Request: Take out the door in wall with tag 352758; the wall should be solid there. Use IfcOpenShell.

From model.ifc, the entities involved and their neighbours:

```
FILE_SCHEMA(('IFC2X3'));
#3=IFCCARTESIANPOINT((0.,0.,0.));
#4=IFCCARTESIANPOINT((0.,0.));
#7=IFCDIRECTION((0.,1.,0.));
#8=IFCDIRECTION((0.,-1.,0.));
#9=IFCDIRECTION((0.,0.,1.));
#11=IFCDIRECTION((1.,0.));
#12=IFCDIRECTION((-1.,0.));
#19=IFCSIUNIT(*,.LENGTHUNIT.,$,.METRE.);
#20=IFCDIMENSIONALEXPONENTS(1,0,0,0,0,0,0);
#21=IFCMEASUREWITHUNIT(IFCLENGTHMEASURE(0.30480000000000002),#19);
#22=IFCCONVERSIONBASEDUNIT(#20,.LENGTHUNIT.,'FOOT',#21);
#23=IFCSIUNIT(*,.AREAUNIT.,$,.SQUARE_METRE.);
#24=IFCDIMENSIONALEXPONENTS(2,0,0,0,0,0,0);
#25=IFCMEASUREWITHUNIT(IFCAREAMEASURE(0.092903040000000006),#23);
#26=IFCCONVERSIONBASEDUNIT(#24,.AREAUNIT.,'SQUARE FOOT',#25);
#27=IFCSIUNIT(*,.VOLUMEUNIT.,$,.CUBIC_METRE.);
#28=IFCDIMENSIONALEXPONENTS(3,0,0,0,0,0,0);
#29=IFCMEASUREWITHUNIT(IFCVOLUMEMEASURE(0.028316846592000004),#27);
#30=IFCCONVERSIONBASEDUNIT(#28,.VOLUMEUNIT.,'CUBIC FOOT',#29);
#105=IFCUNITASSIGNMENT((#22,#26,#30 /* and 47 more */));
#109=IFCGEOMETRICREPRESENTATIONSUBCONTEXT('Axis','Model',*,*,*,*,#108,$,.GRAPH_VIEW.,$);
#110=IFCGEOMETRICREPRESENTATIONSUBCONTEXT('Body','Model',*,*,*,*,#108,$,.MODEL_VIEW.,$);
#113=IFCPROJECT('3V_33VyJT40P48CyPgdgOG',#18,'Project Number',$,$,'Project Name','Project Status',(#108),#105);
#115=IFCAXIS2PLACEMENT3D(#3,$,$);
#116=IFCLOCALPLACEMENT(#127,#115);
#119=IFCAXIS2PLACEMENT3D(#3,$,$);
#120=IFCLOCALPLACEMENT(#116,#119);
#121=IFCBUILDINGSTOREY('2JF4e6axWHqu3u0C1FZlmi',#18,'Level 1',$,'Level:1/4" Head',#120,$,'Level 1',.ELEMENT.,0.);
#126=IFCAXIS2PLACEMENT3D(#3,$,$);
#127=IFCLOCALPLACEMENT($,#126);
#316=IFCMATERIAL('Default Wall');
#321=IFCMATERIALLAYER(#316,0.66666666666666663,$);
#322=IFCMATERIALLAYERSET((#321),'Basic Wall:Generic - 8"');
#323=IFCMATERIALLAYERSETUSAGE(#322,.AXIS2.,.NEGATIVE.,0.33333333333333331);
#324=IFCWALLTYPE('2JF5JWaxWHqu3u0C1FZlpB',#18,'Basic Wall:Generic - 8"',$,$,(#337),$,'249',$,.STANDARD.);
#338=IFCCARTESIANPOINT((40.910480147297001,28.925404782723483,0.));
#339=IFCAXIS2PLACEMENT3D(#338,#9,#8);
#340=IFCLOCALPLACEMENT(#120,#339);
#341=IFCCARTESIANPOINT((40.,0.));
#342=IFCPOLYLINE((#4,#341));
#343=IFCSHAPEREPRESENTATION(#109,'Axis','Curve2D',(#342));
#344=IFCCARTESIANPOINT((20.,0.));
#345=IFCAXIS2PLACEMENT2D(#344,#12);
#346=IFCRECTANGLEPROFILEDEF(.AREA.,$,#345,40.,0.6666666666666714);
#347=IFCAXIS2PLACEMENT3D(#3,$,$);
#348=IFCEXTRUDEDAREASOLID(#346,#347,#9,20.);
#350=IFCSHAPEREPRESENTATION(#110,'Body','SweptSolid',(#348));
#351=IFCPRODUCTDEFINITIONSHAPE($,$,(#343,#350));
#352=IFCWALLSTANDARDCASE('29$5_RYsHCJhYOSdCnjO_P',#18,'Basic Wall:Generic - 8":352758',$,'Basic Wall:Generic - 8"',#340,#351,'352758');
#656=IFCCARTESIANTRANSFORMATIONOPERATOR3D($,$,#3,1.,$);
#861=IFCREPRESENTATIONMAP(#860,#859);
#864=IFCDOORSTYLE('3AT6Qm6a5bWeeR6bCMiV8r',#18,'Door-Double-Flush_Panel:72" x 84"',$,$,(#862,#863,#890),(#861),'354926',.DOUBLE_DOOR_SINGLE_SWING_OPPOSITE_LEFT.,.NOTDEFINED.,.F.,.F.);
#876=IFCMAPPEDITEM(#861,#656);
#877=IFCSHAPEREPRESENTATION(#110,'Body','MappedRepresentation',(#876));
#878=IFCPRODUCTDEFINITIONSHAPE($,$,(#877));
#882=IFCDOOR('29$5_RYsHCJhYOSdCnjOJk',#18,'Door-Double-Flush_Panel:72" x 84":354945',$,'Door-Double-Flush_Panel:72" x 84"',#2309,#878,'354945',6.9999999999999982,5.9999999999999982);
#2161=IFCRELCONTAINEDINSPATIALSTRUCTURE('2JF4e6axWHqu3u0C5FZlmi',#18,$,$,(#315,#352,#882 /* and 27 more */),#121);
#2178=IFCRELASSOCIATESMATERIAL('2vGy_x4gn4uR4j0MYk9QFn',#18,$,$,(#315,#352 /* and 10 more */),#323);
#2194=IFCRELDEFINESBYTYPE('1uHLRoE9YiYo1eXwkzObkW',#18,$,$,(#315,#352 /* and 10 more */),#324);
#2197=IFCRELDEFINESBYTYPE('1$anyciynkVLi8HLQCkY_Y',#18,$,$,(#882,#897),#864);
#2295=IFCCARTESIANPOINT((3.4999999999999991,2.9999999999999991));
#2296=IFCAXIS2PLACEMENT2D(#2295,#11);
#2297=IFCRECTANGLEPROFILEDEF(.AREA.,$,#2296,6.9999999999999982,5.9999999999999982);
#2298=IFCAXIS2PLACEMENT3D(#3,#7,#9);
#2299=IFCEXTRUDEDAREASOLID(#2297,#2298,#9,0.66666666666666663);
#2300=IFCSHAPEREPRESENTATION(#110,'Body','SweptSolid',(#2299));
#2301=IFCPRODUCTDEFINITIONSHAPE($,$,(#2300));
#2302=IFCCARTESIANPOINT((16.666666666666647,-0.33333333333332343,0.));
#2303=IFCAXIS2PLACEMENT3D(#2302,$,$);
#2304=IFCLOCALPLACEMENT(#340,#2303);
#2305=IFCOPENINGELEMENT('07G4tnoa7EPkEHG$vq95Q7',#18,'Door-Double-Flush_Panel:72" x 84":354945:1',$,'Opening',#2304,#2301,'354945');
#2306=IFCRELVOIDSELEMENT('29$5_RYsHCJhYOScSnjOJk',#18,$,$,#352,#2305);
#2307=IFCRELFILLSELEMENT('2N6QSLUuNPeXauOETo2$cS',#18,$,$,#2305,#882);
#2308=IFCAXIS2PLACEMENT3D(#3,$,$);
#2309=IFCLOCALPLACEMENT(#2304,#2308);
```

```python
import ifcopenshell
import ifcopenshell.api.feature
import ifcopenshell.api.root
import ifcopenshell.geom
import ifcopenshell.util.shape

model = ifcopenshell.open("model.ifc")
settings = ifcopenshell.geom.settings()


def volume(element):
    """Net volume in cubic metres, openings subtracted."""
    shape = ifcopenshell.geom.create_shape(settings, element)
    return ifcopenshell.util.shape.get_volume(shape.geometry)


door = model.by_id(882)
opening = door.FillsVoids[0].RelatingOpeningElement
wall = opening.VoidsElements[0].RelatingBuildingElement
before = volume(wall)

ifcopenshell.api.root.remove_product(model, product=door)
ifcopenshell.api.feature.remove_feature(model, feature=opening)

after = volume(wall)

print(f"wall volume {before:.3f} -> {after:.3f} m3")

model.write("model_rev.ifc")
```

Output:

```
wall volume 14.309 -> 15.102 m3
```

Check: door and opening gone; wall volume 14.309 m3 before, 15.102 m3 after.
